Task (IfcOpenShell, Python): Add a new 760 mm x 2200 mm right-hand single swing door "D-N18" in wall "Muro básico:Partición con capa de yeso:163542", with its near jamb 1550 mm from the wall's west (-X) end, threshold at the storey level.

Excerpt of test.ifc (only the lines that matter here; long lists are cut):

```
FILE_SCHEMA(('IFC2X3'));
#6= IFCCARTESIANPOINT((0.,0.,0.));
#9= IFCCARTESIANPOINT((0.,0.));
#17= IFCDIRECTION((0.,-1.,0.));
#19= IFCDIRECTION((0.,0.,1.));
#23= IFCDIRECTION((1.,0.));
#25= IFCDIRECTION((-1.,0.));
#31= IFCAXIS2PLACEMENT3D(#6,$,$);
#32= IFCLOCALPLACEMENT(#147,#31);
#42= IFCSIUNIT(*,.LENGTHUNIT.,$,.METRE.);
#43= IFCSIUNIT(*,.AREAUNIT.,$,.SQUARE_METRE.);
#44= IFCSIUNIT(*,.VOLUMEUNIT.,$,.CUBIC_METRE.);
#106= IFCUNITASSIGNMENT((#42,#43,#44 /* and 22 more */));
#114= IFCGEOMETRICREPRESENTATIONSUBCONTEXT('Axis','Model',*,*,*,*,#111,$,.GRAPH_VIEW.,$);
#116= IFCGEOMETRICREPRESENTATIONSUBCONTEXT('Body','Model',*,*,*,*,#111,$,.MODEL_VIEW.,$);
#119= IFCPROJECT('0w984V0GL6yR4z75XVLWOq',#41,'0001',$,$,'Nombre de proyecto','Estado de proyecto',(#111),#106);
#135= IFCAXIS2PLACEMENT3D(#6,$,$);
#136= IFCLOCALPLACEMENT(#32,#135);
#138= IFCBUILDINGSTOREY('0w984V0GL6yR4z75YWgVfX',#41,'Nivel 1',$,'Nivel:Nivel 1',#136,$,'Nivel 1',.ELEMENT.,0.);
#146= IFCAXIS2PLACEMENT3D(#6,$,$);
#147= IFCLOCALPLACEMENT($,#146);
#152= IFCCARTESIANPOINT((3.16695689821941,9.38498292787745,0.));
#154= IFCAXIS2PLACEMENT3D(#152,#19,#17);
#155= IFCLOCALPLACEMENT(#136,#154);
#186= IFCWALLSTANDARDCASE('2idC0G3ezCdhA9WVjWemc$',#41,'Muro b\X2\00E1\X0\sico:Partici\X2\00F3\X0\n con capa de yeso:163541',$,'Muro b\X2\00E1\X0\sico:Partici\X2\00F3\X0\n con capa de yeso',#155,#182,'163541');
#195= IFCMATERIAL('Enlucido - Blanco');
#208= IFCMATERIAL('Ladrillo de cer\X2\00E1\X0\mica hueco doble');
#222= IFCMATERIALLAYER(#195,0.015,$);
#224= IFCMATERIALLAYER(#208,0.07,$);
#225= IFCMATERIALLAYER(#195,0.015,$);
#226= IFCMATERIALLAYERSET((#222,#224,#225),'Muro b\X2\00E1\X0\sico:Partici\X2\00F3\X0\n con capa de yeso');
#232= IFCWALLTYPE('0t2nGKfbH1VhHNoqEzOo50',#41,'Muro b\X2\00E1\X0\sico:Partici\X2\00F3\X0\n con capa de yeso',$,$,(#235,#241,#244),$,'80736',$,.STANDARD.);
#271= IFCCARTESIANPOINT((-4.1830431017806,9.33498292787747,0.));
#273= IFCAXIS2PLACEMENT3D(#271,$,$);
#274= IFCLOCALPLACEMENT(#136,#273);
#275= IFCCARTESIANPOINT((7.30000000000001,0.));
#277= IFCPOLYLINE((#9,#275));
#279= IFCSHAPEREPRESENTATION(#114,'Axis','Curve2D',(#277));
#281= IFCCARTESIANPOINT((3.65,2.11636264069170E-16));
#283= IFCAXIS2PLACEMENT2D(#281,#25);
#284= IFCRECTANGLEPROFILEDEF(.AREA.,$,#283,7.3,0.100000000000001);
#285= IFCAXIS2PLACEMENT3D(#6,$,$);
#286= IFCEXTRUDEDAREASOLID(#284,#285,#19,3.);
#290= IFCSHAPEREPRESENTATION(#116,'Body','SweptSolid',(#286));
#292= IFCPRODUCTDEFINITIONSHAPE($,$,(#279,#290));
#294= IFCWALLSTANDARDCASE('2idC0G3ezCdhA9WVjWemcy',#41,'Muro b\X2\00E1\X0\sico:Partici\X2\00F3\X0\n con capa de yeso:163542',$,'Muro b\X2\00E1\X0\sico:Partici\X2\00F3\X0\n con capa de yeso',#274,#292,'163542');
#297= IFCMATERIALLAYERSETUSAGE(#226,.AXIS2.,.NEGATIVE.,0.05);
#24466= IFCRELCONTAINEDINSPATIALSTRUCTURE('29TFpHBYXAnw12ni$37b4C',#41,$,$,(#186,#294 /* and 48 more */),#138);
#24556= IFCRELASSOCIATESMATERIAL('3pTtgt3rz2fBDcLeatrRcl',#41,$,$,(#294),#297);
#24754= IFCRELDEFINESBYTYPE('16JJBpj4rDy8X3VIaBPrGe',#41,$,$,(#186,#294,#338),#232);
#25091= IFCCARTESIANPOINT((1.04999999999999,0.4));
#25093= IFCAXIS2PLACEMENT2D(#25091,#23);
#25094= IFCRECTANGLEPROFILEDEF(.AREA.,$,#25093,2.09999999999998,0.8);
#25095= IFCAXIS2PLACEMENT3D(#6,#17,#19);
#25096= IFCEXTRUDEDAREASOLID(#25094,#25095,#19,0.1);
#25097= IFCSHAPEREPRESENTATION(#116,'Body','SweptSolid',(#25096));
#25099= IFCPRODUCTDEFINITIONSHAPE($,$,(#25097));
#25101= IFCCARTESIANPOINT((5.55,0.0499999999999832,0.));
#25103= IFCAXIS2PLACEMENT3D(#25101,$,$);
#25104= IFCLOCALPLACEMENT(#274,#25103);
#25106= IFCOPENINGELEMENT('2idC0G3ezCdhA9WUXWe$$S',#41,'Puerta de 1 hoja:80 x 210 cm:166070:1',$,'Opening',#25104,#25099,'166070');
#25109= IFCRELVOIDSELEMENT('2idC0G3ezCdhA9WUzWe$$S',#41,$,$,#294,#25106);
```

```python
import numpy as np
import ifcopenshell
import ifcopenshell.api.feature
import ifcopenshell.api.geometry
import ifcopenshell.api.root
import ifcopenshell.api.spatial
import ifcopenshell.api.type
import ifcopenshell.geom
import ifcopenshell.util.element
import ifcopenshell.util.placement
import ifcopenshell.util.representation
import ifcopenshell.util.shape
import ifcopenshell.util.unit

model = ifcopenshell.open("test.ifc")
unit_scale = ifcopenshell.util.unit.calculate_unit_scale(model)
settings = ifcopenshell.geom.settings()


def volume(element):
    """Net volume in cubic metres, openings subtracted."""
    shape = ifcopenshell.geom.create_shape(settings, element)
    return ifcopenshell.util.shape.get_volume(shape.geometry)


wall = model.by_guid("2idC0G3ezCdhA9WVjWemcy")
storey = ifcopenshell.util.element.get_container(wall, ifc_class="IfcBuildingStorey")
context = ifcopenshell.util.representation.get_context(model, "Model", "Body", "MODEL_VIEW")
before = volume(wall)

width, height, from_end, sill = 0.76, 2.2, 1.55, 0.0  # metres

# The wall runs along its own X axis, and the end named is its -X end.
wall_shape = ifcopenshell.geom.create_shape(settings, wall)
x, y, z = ifcopenshell.util.shape.get_vertices(wall_shape.geometry).T
start = x.min() + from_end
face, thickness = float(y.min()), float(y.max() - y.min())
wall_matrix = ifcopenshell.util.placement.get_local_placement(wall.ObjectPlacement)
level = ifcopenshell.util.placement.get_local_placement(storey.ObjectPlacement)[2, 3]


def in_wall(x, y):
    """Placement at x, y metres in the wall's axes, at sill height."""
    matrix = wall_matrix.copy()
    matrix[:, 3] = wall_matrix @ np.array([x / unit_scale, y / unit_scale, 0.0, 1.0])
    matrix[2, 3] = level + sill / unit_scale
    return matrix


# Opening: a box that overshoots both wall faces by 50 mm.
opening = ifcopenshell.api.root.create_entity(model, ifc_class="IfcOpeningElement")
box = ifcopenshell.api.geometry.add_wall_representation(
    model, context=context, length=width, height=height, thickness=thickness + 0.1
)
ifcopenshell.api.geometry.assign_representation(model, product=opening, representation=box)
ifcopenshell.api.geometry.edit_object_placement(model, product=opening, matrix=in_wall(start, face - 0.05), is_si=False)
ifcopenshell.api.feature.add_feature(model, feature=opening, element=wall)

door = ifcopenshell.api.root.create_entity(model, ifc_class="IfcDoor", name="D-N18")
door.OverallWidth, door.OverallHeight = width / unit_scale, height / unit_scale
body = ifcopenshell.api.geometry.add_door_representation(
    model,
    context=context,
    overall_width=door.OverallWidth,
    overall_height=door.OverallHeight,
    operation_type="SINGLE_SWING_RIGHT",
    lining_properties={"LiningDepth": thickness / unit_scale, "ThresholdDepth": thickness / unit_scale},
)
ifcopenshell.api.geometry.assign_representation(model, product=door, representation=body)
ifcopenshell.api.spatial.assign_container(model, products=[door], relating_structure=storey)
fills = ifcopenshell.api.feature.add_filling(model, opening=opening, element=door)
fills.OwnerHistory = door.OwnerHistory  # required in IFC2X3

# IFC2X3 keeps the operation on the door style.
style = ifcopenshell.api.root.create_entity(model, ifc_class="IfcDoorStyle", name="D-N18")
style.OperationType, style.ConstructionType = "SINGLE_SWING_RIGHT", "NOTDEFINED"
style.ParameterTakesPrecedence = style.Sizeable = False
ifcopenshell.api.type.assign_type(model, related_objects=[door], relating_type=style)

# The lining spans the wall, so the door starts at the wall face.
ifcopenshell.api.geometry.edit_object_placement(model, product=door, matrix=in_wall(start, face), is_si=False)

after = volume(wall)

print(f"wall volume {before:.3f} -> {after:.3f} m3")

model.write("test-out.ifc")
```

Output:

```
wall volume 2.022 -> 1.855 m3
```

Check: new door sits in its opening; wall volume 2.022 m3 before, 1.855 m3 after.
